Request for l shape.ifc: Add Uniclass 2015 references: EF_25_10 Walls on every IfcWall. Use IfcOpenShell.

First a look at what the model holds.

```python
import ifcopenshell

model = ifcopenshell.open("l shape.ifc")
print(model.schema)
print("classifications:", [c.Name for c in model.by_type("IfcClassification")])
for ifc_class in ("IfcDoor", "IfcRoof", "IfcStair", "IfcWall", "IfcWindow"):
    print(ifc_class, len(model.by_type(ifc_class)))
```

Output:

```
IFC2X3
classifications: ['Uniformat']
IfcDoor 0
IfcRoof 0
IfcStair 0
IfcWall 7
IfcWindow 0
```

```python
import ifcopenshell
import ifcopenshell.api.classification

model = ifcopenshell.open("l shape.ifc")

# IFC2X3 requires Source and Edition and has no link from the project to the system.
system = model.create_entity("IfcClassification", Source="NBS", Edition="2015", Name="Uniclass 2015")

codes = {
    "IfcWall": ("EF_25_10", "Walls"),
}
for ifc_class, (code, name) in codes.items():
    products = model.by_type(ifc_class)
    ifcopenshell.api.classification.add_reference(
        model, products=products, classification=system, identification=code, name=name
    )
    print(code, len(products))

model.write("l shape_updated.ifc")
```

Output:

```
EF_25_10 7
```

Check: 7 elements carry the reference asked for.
